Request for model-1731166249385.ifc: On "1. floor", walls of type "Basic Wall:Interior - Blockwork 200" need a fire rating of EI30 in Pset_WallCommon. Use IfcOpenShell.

First a look at what the model holds.

```python
import ifcopenshell
import ifcopenshell.util.element

model = ifcopenshell.open("model-1731166249385.ifc")
print(model.schema)
storey = next(s for s in model.by_type("IfcBuildingStorey") if s.Name == "1. floor")
walls = [e for e in ifcopenshell.util.element.get_decomposition(storey) if e.is_a("IfcWall")]
seen = {}
for e in walls:
    element_type = ifcopenshell.util.element.get_type(e)
    key = (element_type.Name if element_type != e and element_type else None, ifcopenshell.util.element.get_pset(e, "Pset_WallCommon", "FireRating"))
    seen[key] = seen.get(key, 0) + 1
for (name, value), count in sorted(seen.items(), key=str):
    print(count, "x", name, "|", value)
```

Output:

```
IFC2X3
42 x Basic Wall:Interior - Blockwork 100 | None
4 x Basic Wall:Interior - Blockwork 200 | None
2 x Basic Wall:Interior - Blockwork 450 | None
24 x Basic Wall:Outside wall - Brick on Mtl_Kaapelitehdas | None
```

```python
import ifcopenshell
import ifcopenshell.api.pset
import ifcopenshell.util.element

model = ifcopenshell.open("model-1731166249385.ifc")

storey = next(s for s in model.by_type("IfcBuildingStorey") if s.Name == "1. floor")
walls = [e for e in ifcopenshell.util.element.get_decomposition(storey) if e.is_a("IfcWall")]

count = 0
for e in walls:
    element_type = ifcopenshell.util.element.get_type(e)
    if element_type in (None, e) or element_type.Name != "Basic Wall:Interior - Blockwork 200":
        continue
    # add_pset returns the element's existing set when there is one.
    pset = ifcopenshell.api.pset.add_pset(model, product=e, name="Pset_WallCommon")
    ifcopenshell.api.pset.edit_pset(model, pset=pset, properties={"FireRating": "EI30"})
    count += 1

print(count, "walls updated")

model.write("model-1731166249385_rev.ifc")
```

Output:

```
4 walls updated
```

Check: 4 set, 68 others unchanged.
